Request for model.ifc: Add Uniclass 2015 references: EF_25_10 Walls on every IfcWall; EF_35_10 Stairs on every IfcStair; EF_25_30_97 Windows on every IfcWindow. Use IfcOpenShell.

First a look at what the model holds.

```python
import ifcopenshell

model = ifcopenshell.open("model.ifc")
print(model.schema)
print("classifications:", [c.Name for c in model.by_type("IfcClassification")])
for ifc_class in ("IfcDoor", "IfcRoof", "IfcStair", "IfcWall", "IfcWindow"):
    print(ifc_class, len(model.by_type(ifc_class)))
```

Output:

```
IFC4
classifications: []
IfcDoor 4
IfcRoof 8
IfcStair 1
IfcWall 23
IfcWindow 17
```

```python
import ifcopenshell
import ifcopenshell.api.classification

model = ifcopenshell.open("model.ifc")

system = ifcopenshell.api.classification.add_classification(model, classification="Uniclass 2015")

codes = {
    "IfcWall": ("EF_25_10", "Walls"),
    "IfcStair": ("EF_35_10", "Stairs"),
    "IfcWindow": ("EF_25_30_97", "Windows"),
}
for ifc_class, (code, name) in codes.items():
    products = model.by_type(ifc_class)
    ifcopenshell.api.classification.add_reference(
        model, products=products, classification=system, identification=code, name=name
    )
    print(code, len(products))

model.write("model_rev.ifc")
```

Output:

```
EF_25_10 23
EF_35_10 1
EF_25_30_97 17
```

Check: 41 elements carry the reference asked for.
